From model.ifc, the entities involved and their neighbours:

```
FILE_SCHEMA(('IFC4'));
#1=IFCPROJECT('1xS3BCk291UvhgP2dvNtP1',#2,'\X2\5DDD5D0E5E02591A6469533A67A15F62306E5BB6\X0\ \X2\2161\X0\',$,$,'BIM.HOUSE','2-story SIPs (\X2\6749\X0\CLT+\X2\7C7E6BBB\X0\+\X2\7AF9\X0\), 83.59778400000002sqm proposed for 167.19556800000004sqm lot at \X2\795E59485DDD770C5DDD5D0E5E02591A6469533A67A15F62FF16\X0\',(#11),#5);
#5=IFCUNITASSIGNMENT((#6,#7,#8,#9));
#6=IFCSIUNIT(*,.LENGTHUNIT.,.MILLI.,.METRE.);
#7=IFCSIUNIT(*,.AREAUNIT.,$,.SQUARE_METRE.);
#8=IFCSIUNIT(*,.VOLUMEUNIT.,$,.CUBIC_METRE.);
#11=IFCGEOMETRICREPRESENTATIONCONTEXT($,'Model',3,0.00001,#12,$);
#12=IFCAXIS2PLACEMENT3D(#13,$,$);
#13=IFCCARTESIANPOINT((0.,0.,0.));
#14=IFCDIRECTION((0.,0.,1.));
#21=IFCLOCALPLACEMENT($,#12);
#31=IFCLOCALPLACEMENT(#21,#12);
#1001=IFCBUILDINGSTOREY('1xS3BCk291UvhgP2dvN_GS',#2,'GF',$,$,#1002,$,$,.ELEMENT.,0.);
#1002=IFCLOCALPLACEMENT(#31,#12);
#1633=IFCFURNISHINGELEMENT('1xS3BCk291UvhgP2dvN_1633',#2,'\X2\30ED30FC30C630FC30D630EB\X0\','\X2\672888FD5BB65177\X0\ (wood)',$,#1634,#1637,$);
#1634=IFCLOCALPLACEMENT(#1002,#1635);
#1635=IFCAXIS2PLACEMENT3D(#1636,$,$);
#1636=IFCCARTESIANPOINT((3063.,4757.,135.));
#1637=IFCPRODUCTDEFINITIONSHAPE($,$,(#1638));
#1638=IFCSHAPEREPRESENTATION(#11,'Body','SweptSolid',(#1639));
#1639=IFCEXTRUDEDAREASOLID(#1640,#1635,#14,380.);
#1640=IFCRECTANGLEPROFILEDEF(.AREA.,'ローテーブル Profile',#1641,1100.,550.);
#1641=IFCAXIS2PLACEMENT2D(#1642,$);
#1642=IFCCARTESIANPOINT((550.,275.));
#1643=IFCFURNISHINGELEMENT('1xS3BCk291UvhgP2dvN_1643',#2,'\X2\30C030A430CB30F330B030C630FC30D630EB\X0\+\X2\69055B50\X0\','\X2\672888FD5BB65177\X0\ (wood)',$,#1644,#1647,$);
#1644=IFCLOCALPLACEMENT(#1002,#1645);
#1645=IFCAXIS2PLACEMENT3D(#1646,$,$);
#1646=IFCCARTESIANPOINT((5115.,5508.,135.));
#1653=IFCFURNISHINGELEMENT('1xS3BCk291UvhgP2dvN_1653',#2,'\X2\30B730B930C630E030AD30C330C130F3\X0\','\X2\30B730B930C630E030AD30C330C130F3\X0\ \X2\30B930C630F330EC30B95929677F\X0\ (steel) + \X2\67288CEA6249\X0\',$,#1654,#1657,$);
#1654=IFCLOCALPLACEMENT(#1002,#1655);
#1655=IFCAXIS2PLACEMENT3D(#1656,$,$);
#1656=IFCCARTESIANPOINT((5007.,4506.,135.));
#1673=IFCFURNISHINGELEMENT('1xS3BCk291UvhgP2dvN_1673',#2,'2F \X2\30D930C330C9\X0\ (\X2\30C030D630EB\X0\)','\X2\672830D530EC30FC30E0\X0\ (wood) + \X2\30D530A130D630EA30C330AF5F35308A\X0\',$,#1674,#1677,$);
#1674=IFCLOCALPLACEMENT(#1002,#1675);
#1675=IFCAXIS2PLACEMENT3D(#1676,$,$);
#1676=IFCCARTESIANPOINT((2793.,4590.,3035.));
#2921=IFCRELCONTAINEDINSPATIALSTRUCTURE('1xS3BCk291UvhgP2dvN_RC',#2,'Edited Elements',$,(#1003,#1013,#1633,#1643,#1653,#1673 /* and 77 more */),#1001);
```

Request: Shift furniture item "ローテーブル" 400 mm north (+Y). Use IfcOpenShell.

```python
import ifcopenshell
import ifcopenshell.api.geometry
import ifcopenshell.util.placement
import ifcopenshell.util.unit

model = ifcopenshell.open("model.ifc")
unit_scale = ifcopenshell.util.unit.calculate_unit_scale(model)

item = model.by_id(1633)
matrix = ifcopenshell.util.placement.get_local_placement(item.ObjectPlacement)
matrix[1, 3] += 0.4 / unit_scale
ifcopenshell.api.geometry.edit_object_placement(model, product=item, matrix=matrix, is_si=False)

print(ifcopenshell.util.placement.get_local_placement(item.ObjectPlacement).round(3) + 0.0)

model.write("model_updated.ifc")
```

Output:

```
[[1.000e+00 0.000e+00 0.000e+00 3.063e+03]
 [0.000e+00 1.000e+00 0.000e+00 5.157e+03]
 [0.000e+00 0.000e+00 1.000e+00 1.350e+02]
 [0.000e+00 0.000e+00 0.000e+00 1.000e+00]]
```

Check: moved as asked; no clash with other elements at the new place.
